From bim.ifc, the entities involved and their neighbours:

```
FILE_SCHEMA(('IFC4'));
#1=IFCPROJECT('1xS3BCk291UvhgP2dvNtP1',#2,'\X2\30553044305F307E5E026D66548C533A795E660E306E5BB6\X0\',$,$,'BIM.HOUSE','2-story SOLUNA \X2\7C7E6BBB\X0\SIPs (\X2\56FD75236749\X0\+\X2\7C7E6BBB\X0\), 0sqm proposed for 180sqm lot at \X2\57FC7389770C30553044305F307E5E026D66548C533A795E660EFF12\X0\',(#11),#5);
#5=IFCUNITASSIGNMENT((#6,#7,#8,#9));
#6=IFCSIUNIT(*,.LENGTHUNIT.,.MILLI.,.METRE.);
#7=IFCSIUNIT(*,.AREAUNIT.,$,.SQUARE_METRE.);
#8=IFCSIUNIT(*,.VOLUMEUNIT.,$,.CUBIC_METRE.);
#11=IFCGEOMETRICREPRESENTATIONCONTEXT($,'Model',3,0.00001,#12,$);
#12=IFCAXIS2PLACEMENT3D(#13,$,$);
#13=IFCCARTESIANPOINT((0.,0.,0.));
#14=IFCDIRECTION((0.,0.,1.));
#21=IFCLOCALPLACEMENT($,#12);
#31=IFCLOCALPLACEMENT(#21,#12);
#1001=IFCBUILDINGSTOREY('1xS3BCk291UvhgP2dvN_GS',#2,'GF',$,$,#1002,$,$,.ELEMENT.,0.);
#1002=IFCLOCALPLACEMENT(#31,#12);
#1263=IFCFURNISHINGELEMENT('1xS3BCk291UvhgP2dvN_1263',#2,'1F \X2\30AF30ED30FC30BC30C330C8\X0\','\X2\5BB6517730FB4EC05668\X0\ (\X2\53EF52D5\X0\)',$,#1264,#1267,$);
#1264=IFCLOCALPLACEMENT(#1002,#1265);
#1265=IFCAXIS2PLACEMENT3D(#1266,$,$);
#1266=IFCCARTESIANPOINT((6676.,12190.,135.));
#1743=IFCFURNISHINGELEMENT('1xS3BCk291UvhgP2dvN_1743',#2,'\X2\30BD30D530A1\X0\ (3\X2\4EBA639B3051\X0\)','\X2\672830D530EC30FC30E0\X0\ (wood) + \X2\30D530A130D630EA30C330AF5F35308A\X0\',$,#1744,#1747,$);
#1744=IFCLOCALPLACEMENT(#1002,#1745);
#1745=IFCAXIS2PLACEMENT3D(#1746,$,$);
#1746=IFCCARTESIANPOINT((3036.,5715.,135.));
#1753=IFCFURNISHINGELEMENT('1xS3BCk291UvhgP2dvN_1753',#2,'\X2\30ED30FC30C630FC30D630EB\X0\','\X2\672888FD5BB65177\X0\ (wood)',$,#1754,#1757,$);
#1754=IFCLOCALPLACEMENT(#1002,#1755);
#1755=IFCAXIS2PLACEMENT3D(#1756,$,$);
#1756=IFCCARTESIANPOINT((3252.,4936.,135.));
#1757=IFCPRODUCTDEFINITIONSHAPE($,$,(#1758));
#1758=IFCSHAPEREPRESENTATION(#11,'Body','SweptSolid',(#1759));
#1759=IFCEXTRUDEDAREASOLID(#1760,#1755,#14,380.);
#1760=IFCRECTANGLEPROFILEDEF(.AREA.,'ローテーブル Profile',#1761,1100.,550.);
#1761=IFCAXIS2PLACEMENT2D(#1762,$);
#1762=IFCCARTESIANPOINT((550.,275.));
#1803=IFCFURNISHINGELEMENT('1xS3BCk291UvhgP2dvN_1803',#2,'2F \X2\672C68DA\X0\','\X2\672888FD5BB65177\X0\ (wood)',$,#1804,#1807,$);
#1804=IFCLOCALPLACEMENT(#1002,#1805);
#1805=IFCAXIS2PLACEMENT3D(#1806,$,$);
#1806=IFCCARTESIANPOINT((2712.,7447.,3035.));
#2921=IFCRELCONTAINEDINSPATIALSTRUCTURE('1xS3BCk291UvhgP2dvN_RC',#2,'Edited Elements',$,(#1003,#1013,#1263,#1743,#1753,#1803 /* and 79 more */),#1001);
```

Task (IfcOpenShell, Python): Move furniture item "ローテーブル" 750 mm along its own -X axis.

```python
import ifcopenshell
import ifcopenshell.api.geometry
import ifcopenshell.util.placement

model = ifcopenshell.open("bim.ifc")

item = model.by_guid("1xS3BCk291UvhgP2dvN_1753")
matrix = ifcopenshell.util.placement.get_local_placement(item.ObjectPlacement)
matrix[:3, 3] -= matrix[:3, 0] * 750.0
ifcopenshell.api.geometry.edit_object_placement(model, product=item, matrix=matrix, is_si=False)

print(ifcopenshell.util.placement.get_local_placement(item.ObjectPlacement).round(3) + 0.0)

model.write("bim-out.ifc")
```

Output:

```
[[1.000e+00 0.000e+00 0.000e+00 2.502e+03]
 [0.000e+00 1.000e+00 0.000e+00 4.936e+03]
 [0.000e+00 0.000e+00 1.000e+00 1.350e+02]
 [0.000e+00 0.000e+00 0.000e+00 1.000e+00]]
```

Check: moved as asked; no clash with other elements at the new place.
